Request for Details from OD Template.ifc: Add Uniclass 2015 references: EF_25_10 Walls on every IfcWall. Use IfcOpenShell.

First a look at what the model holds.

```python
import ifcopenshell

model = ifcopenshell.open("Details from OD Template.ifc")
print(model.schema)
print("classifications:", [c.Name for c in model.by_type("IfcClassification")])
for ifc_class in ("IfcDoor", "IfcRoof", "IfcStair", "IfcWall", "IfcWindow"):
    print(ifc_class, len(model.by_type(ifc_class)))
```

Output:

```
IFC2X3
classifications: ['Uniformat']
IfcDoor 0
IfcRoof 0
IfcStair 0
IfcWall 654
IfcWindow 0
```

```python
import ifcopenshell
import ifcopenshell.api.classification

model = ifcopenshell.open("Details from OD Template.ifc")

# IFC2X3 requires Source and Edition and has no link from the project to the system.
system = model.create_entity("IfcClassification", Source="NBS", Edition="2015", Name="Uniclass 2015")

codes = {
    "IfcWall": ("EF_25_10", "Walls"),
}
for ifc_class, (code, name) in codes.items():
    products = model.by_type(ifc_class)
    ifcopenshell.api.classification.add_reference(
        model, products=products, classification=system, identification=code, name=name
    )
    print(code, len(products))

model.write("Details from OD Template_rev.ifc")
```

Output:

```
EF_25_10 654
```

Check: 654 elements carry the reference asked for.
